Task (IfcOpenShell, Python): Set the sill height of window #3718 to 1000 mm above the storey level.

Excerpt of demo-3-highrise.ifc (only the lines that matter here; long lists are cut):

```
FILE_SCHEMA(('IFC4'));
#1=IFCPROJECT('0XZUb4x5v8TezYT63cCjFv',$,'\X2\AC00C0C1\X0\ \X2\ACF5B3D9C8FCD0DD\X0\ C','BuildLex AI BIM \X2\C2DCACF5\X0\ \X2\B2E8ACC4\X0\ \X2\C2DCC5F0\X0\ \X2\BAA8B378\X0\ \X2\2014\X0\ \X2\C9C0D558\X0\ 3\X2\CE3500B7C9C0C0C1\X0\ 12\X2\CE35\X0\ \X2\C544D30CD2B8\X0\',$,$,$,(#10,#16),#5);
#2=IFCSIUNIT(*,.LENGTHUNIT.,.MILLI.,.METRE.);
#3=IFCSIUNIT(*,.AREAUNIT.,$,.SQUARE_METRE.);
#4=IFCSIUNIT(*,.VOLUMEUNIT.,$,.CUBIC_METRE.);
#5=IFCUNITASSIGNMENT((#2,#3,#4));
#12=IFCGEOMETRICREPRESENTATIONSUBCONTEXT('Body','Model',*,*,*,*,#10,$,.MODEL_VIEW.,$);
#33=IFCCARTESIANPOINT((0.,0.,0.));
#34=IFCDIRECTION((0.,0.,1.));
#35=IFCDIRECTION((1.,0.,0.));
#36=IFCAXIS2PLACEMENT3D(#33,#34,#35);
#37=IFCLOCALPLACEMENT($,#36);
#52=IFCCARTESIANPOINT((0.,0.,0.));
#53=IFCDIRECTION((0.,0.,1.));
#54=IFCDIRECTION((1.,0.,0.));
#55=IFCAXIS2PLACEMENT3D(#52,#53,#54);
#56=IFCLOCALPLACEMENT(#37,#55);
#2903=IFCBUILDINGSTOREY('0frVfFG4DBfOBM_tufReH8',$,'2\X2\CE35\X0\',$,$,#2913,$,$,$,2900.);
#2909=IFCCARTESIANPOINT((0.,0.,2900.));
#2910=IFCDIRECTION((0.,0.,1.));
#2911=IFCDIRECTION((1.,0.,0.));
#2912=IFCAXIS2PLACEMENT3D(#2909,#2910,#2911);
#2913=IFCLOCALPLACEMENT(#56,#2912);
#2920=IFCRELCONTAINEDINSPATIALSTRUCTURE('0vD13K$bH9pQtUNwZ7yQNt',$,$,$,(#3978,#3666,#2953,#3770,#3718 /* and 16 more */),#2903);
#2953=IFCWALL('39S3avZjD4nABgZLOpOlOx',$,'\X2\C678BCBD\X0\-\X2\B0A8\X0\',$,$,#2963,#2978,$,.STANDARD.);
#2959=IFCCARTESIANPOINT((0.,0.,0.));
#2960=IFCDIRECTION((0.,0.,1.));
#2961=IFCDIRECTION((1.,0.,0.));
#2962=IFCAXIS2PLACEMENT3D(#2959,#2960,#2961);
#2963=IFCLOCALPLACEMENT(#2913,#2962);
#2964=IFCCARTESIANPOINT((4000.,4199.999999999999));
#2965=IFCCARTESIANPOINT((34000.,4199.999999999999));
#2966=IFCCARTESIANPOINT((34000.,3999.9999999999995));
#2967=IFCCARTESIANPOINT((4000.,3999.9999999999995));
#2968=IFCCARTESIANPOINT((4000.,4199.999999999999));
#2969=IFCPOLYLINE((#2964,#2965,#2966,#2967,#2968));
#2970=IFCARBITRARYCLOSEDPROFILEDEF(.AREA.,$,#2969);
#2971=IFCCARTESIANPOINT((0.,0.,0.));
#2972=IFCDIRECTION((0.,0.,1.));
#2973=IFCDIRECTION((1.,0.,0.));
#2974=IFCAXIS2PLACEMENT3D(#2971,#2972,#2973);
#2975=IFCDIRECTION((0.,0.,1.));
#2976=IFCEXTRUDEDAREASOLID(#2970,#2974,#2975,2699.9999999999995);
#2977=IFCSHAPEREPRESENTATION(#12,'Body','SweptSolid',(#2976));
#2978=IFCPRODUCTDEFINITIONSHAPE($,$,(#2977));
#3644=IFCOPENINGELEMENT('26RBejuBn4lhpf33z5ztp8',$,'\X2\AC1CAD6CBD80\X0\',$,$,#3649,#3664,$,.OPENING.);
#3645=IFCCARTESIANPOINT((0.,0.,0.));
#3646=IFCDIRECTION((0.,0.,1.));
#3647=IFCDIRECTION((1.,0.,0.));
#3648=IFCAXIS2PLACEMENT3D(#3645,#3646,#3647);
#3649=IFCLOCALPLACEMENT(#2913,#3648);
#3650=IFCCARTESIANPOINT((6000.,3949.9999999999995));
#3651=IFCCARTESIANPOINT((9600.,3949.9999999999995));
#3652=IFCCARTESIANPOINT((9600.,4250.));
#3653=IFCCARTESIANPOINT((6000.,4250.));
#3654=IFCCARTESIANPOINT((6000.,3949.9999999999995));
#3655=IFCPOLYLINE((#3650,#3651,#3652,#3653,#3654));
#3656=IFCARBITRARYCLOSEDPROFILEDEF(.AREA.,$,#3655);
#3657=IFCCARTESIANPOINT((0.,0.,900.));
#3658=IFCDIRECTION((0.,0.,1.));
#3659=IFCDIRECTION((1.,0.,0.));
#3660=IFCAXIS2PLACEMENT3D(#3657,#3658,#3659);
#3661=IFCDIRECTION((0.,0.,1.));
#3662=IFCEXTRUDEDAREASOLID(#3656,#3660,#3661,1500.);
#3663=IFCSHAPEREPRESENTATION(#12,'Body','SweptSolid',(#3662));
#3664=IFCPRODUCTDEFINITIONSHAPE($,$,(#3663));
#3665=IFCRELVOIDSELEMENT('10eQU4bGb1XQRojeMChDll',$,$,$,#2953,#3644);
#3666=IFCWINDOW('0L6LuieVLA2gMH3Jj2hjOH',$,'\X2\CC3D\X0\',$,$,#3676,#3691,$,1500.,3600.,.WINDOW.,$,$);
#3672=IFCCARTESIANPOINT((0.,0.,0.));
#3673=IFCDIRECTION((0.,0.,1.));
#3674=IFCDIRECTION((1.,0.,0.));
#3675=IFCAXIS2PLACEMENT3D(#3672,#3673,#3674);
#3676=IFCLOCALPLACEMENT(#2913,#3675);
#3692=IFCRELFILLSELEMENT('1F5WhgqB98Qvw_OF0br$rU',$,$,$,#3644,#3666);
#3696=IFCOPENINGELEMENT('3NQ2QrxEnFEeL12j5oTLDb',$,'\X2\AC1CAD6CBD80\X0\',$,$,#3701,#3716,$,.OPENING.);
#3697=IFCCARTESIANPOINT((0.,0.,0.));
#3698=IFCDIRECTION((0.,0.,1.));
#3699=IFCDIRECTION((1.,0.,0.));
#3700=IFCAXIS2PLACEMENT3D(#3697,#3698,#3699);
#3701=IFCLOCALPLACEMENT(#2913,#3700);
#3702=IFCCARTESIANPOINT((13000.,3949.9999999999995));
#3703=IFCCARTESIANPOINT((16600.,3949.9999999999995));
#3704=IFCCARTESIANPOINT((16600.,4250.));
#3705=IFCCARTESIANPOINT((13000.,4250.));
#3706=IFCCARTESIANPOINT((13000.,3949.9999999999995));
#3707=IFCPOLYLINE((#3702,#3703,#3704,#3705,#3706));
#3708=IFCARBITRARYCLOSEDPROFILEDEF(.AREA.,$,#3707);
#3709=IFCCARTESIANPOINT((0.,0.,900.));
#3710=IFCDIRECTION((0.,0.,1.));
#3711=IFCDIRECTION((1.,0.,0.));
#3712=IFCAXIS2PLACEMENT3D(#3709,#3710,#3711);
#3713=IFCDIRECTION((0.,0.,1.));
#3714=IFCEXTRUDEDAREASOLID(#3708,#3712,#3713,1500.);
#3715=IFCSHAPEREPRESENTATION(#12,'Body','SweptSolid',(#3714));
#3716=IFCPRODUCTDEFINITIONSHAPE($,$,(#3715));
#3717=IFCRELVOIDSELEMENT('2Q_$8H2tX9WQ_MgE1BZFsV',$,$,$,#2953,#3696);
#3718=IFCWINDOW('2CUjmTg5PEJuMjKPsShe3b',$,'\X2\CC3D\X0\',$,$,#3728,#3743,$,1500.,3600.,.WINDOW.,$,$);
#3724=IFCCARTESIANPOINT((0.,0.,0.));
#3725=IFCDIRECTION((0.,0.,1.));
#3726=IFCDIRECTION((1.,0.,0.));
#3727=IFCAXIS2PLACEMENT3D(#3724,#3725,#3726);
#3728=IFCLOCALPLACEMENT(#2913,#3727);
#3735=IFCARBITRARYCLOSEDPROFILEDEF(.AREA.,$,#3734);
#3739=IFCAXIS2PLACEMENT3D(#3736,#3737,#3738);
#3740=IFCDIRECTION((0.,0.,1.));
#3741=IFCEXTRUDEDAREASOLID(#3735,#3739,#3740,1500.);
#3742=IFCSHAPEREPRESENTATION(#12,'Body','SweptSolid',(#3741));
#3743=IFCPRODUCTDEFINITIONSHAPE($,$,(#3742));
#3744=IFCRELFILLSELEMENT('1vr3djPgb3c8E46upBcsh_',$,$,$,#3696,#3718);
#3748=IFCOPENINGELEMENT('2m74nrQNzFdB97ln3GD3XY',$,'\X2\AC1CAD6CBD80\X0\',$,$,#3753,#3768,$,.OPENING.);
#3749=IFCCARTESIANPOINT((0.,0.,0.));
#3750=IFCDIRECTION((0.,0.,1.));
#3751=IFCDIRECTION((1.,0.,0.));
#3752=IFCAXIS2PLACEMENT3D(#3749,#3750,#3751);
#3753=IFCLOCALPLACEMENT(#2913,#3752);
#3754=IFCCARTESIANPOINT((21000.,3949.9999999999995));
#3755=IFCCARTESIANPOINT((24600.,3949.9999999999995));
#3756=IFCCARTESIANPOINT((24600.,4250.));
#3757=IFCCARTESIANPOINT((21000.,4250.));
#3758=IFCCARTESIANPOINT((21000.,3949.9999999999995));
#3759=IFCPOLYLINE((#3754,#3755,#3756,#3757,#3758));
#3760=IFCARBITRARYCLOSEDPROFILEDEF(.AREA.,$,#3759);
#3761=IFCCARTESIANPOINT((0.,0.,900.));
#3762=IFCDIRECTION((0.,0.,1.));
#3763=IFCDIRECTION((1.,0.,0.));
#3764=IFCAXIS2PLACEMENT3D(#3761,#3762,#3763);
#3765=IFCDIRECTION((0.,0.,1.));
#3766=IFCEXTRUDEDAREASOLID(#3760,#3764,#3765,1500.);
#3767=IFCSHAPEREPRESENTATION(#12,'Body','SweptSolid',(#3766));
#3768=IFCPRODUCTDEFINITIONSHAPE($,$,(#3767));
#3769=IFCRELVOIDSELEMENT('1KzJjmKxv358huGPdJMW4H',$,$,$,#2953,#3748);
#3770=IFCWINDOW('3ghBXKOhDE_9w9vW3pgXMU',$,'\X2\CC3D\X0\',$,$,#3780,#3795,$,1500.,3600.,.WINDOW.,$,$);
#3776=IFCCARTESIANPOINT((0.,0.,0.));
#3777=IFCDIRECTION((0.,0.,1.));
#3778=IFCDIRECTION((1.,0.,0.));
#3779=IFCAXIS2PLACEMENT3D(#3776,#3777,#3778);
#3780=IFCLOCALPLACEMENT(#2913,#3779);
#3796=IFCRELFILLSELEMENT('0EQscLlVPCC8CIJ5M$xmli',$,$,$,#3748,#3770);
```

```python
import numpy as np
import ifcopenshell
import ifcopenshell.api.geometry
import ifcopenshell.geom
import ifcopenshell.util.element
import ifcopenshell.util.placement
import ifcopenshell.util.shape
import ifcopenshell.util.unit

model = ifcopenshell.open("demo-3-highrise.ifc")
unit_scale = ifcopenshell.util.unit.calculate_unit_scale(model)

window = model.by_guid("2CUjmTg5PEJuMjKPsShe3b")
opening = window.FillsVoids[0].RelatingOpeningElement
storey = ifcopenshell.util.element.get_container(window, ifc_class="IfcBuildingStorey")
level = ifcopenshell.util.placement.get_local_placement(storey.ObjectPlacement)[2, 3]

# The opening's origin need not be at the sill, so measure its lowest point.
shape = ifcopenshell.geom.create_shape(ifcopenshell.geom.settings(), opening)
bottom = ifcopenshell.util.shape.get_shape_bottom_elevation(shape, shape.geometry) / unit_scale
dz = level + 1 / unit_scale - bottom

shift = np.array([0.0, 0.0, dz])
# The window is not placed relative to its opening, so move both.
for product in (opening, window):
    matrix = ifcopenshell.util.placement.get_local_placement(product.ObjectPlacement)
    matrix[:3, 3] += shift
    ifcopenshell.api.geometry.edit_object_placement(model, product=product, matrix=matrix, is_si=False)

print(f"moved by {dz * unit_scale:+.3f} m")

model.write("demo-3-highrise_rev.ifc")
```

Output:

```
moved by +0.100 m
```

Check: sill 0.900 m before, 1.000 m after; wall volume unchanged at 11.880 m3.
